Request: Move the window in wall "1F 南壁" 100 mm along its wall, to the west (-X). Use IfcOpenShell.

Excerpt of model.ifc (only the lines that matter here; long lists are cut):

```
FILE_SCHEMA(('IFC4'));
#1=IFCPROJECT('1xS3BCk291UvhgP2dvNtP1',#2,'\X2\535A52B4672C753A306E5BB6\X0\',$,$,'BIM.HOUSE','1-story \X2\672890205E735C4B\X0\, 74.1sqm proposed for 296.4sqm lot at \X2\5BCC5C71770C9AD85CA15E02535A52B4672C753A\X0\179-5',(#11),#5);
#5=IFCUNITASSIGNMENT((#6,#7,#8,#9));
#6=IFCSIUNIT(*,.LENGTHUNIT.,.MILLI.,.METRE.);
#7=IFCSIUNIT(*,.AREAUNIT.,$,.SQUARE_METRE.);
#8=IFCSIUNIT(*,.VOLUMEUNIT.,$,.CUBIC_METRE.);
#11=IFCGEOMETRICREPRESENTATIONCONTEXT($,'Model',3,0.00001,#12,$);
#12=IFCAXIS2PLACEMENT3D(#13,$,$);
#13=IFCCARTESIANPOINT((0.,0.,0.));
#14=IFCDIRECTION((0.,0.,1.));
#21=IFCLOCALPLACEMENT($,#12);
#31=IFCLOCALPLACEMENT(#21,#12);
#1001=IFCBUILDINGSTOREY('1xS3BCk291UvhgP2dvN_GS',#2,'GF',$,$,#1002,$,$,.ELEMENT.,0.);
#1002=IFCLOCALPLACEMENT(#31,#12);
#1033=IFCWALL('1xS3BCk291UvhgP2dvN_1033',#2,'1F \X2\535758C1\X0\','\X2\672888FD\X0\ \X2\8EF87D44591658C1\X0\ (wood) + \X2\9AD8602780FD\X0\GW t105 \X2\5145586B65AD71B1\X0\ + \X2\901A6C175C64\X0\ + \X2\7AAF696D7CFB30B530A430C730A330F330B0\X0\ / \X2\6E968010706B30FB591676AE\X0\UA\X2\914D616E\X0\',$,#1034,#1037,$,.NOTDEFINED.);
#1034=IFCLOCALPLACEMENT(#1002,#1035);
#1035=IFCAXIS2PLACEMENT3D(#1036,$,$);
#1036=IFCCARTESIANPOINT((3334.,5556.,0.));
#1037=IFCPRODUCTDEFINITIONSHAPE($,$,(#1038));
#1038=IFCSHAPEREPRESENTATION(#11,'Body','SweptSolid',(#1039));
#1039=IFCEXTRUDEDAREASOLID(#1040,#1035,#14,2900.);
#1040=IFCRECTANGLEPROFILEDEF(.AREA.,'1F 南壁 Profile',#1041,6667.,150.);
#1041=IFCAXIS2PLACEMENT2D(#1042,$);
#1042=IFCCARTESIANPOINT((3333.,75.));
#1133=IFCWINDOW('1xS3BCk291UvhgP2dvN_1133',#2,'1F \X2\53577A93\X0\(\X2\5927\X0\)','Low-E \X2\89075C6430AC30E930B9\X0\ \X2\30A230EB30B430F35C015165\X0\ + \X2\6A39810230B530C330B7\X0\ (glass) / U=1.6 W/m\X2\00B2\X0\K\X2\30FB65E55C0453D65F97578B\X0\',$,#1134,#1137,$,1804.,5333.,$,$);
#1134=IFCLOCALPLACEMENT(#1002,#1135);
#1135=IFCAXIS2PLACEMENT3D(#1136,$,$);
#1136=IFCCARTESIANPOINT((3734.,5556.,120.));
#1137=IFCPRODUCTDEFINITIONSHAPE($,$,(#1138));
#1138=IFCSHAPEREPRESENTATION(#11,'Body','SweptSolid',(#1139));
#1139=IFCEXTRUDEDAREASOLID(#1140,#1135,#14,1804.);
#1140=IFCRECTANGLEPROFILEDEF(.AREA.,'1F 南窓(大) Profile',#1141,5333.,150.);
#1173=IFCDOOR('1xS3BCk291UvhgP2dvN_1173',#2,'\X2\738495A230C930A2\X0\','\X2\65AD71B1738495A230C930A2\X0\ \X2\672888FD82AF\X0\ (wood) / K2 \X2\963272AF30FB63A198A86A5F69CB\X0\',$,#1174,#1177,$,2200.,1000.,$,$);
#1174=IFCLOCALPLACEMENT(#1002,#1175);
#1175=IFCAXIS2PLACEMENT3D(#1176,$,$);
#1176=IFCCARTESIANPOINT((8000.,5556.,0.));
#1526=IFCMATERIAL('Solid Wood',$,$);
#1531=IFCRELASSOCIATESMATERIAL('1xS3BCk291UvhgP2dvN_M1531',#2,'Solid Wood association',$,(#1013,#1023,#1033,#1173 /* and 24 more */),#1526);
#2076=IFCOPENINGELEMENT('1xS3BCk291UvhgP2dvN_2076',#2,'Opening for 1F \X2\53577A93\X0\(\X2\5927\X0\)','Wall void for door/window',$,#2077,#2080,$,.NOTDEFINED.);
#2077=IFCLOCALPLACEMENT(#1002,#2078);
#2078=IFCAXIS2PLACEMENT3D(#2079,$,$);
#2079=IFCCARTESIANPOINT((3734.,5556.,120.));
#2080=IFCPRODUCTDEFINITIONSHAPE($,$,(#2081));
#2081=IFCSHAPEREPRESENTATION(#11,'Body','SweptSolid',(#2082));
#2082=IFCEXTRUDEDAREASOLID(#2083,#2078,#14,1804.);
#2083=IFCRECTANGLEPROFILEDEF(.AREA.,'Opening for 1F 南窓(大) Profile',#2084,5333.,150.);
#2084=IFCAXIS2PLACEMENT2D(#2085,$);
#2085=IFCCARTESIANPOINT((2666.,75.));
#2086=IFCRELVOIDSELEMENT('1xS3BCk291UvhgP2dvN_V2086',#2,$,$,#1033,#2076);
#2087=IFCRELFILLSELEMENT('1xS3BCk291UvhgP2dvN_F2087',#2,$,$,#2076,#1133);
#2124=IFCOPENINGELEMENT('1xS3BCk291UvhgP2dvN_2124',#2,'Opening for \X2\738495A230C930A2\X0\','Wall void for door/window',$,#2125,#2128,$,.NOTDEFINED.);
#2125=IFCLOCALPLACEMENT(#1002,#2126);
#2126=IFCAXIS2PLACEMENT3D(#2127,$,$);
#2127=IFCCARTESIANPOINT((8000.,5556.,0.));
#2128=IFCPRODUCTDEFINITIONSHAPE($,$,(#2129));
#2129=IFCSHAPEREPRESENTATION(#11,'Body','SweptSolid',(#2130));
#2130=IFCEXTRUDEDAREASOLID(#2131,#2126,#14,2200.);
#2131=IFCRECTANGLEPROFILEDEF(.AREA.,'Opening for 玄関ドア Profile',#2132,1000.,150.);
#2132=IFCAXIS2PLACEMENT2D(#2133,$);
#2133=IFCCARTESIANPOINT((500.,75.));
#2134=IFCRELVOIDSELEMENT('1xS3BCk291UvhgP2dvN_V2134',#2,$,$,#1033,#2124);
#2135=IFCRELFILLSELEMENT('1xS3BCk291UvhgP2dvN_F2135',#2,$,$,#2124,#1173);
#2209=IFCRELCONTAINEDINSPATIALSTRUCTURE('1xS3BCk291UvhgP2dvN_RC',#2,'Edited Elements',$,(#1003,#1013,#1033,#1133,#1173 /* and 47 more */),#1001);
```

```python
import ifcopenshell
import ifcopenshell.api.geometry
import ifcopenshell.util.placement
import ifcopenshell.util.unit

model = ifcopenshell.open("model.ifc")
unit_scale = ifcopenshell.util.unit.calculate_unit_scale(model)

window = model.by_guid("1xS3BCk291UvhgP2dvN_1133")
opening = window.FillsVoids[0].RelatingOpeningElement
wall = opening.VoidsElements[0].RelatingBuildingElement

wall_matrix = ifcopenshell.util.placement.get_local_placement(wall.ObjectPlacement)
shift = wall_matrix[:3, 0] * -0.1 / unit_scale
before = ifcopenshell.util.placement.get_local_placement(window.ObjectPlacement)[:3, 3].copy()

# The window is not placed relative to its opening, so move both.
for product in (opening, window):
    matrix = ifcopenshell.util.placement.get_local_placement(product.ObjectPlacement)
    matrix[:3, 3] += shift
    ifcopenshell.api.geometry.edit_object_placement(model, product=product, matrix=matrix, is_si=False)

after = ifcopenshell.util.placement.get_local_placement(window.ObjectPlacement)[:3, 3]
print("window moved by", (after - before).round(3) + 0.0)

model.write("model-out.ifc")
```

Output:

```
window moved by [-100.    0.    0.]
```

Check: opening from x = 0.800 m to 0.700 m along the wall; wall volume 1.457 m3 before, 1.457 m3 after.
